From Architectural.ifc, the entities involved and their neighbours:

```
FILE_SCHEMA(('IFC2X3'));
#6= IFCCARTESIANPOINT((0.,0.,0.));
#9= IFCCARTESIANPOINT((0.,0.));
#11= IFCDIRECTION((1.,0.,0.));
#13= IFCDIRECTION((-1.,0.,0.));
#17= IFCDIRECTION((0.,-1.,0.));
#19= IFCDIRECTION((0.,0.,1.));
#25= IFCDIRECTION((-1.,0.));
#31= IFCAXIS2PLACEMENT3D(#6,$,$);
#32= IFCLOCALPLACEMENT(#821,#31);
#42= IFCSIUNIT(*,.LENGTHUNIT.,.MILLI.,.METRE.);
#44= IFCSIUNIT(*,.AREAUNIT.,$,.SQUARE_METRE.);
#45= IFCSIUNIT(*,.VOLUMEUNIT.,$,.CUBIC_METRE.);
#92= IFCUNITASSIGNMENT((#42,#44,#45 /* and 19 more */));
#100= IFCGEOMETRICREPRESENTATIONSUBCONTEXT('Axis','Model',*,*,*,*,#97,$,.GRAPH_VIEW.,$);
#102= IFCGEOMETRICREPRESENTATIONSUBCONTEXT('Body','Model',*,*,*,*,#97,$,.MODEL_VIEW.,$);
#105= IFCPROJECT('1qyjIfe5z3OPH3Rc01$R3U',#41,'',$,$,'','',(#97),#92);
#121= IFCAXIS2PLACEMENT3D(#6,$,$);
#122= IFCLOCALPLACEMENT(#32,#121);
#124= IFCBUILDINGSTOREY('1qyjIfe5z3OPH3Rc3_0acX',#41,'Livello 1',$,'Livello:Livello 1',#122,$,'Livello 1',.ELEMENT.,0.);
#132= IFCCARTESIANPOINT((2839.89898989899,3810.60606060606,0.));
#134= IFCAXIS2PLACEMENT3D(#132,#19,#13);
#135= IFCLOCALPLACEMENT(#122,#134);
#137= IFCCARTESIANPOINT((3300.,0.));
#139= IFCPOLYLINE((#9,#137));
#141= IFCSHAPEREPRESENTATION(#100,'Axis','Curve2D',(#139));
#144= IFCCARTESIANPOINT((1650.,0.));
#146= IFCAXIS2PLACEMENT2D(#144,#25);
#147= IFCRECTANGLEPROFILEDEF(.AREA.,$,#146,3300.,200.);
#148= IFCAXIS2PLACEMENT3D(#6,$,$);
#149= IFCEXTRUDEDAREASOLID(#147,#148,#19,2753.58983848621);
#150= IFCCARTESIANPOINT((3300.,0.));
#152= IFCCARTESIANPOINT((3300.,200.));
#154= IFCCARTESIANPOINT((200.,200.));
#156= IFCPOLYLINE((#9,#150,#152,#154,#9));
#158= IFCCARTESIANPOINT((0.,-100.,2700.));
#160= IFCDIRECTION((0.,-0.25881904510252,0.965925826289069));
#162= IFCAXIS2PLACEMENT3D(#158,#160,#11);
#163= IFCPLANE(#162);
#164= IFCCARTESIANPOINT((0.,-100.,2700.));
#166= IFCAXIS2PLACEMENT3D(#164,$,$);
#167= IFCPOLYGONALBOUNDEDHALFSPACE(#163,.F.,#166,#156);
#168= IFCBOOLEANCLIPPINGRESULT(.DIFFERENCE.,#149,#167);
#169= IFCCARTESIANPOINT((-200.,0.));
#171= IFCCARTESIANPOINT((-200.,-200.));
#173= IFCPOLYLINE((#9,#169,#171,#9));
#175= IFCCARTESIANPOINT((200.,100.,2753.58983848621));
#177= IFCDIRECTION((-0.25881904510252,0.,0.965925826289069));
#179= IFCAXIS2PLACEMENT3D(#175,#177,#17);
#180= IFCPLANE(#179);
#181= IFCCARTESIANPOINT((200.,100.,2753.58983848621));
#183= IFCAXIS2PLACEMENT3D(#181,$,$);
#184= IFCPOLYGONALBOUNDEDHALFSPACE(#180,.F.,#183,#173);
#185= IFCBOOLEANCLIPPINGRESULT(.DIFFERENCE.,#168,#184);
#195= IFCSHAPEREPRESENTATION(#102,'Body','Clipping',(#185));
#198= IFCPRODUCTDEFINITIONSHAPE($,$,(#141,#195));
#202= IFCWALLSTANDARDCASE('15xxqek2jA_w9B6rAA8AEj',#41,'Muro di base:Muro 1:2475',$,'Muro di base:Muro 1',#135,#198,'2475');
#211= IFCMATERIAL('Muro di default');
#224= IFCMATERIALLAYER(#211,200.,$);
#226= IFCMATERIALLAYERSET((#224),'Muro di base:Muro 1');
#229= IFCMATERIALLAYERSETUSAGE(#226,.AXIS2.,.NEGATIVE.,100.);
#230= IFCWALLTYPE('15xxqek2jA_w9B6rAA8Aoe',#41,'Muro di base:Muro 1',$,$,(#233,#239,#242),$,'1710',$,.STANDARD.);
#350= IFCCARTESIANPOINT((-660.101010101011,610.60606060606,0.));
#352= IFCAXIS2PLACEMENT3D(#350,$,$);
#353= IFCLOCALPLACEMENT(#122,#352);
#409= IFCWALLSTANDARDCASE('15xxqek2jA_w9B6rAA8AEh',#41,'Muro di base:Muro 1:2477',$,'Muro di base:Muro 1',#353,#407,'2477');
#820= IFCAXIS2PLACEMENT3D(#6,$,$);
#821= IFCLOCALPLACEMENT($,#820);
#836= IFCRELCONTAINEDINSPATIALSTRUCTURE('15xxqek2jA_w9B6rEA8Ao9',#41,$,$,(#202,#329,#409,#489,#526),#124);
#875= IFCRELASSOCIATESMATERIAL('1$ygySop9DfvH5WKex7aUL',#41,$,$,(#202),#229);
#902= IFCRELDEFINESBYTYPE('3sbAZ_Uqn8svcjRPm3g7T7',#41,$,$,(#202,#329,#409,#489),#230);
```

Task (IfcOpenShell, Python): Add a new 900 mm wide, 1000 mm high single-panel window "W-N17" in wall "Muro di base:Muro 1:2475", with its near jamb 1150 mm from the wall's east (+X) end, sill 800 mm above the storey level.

```python
import numpy as np
import ifcopenshell
import ifcopenshell.api.feature
import ifcopenshell.api.geometry
import ifcopenshell.api.root
import ifcopenshell.api.spatial
import ifcopenshell.api.type
import ifcopenshell.geom
import ifcopenshell.util.element
import ifcopenshell.util.placement
import ifcopenshell.util.representation
import ifcopenshell.util.shape
import ifcopenshell.util.unit

model = ifcopenshell.open("Architectural.ifc")
unit_scale = ifcopenshell.util.unit.calculate_unit_scale(model)
settings = ifcopenshell.geom.settings()


def volume(element):
    """Net volume in cubic metres, openings subtracted."""
    shape = ifcopenshell.geom.create_shape(settings, element)
    return ifcopenshell.util.shape.get_volume(shape.geometry)


wall = model.by_id(202)
storey = ifcopenshell.util.element.get_container(wall, ifc_class="IfcBuildingStorey")
context = ifcopenshell.util.representation.get_context(model, "Model", "Body", "MODEL_VIEW")
before = volume(wall)

width, height, from_end, sill = 0.9, 1, 1.15, 0.8  # metres

# The wall runs along its own X axis, and the end named is its -X end.
wall_shape = ifcopenshell.geom.create_shape(settings, wall)
x, y, z = ifcopenshell.util.shape.get_vertices(wall_shape.geometry).T
start = x.min() + from_end
face, thickness = float(y.min()), float(y.max() - y.min())
wall_matrix = ifcopenshell.util.placement.get_local_placement(wall.ObjectPlacement)
level = ifcopenshell.util.placement.get_local_placement(storey.ObjectPlacement)[2, 3]


def in_wall(x, y):
    """Placement at x, y metres in the wall's axes, at sill height."""
    matrix = wall_matrix.copy()
    matrix[:, 3] = wall_matrix @ np.array([x / unit_scale, y / unit_scale, 0.0, 1.0])
    matrix[2, 3] = level + sill / unit_scale
    return matrix


# Opening: a box that overshoots both wall faces by 50 mm.
opening = ifcopenshell.api.root.create_entity(model, ifc_class="IfcOpeningElement")
box = ifcopenshell.api.geometry.add_wall_representation(
    model, context=context, length=width, height=height, thickness=thickness + 0.1
)
ifcopenshell.api.geometry.assign_representation(model, product=opening, representation=box)
ifcopenshell.api.geometry.edit_object_placement(model, product=opening, matrix=in_wall(start, face - 0.05), is_si=False)
ifcopenshell.api.feature.add_feature(model, feature=opening, element=wall)

window = ifcopenshell.api.root.create_entity(model, ifc_class="IfcWindow", name="W-N17")
window.OverallWidth, window.OverallHeight = width / unit_scale, height / unit_scale
body = ifcopenshell.api.geometry.add_window_representation(
    model,
    context=context,
    overall_width=window.OverallWidth,
    overall_height=window.OverallHeight,
    partition_type="SINGLE_PANEL",
)
ifcopenshell.api.geometry.assign_representation(model, product=window, representation=body)
ifcopenshell.api.spatial.assign_container(model, products=[window], relating_structure=storey)
fills = ifcopenshell.api.feature.add_filling(model, opening=opening, element=window)
fills.OwnerHistory = window.OwnerHistory  # required in IFC2X3

# IFC2X3 keeps the operation on the window style.
style = ifcopenshell.api.root.create_entity(model, ifc_class="IfcWindowStyle", name="W-N17")
style.OperationType, style.ConstructionType = "SINGLE_PANEL", "NOTDEFINED"
style.ParameterTakesPrecedence = style.Sizeable = False
ifcopenshell.api.type.assign_type(model, related_objects=[window], relating_type=style)

# Centre the window in the wall's thickness.
ifcopenshell.api.geometry.edit_object_placement(model, product=window, matrix=in_wall(start, face), is_si=False)
window_shape = ifcopenshell.geom.create_shape(settings, window)
depth = ifcopenshell.util.shape.get_vertices(window_shape.geometry)[:, 1]
offset = face + thickness / 2 - (depth.min() + depth.max()) / 2
ifcopenshell.api.geometry.edit_object_placement(model, product=window, matrix=in_wall(start, offset), is_si=False)

after = volume(wall)

print(f"wall volume {before:.3f} -> {after:.3f} m3")

model.write("Architectural_edited.ifc")
```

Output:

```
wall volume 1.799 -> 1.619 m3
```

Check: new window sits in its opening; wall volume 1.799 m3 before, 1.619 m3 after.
